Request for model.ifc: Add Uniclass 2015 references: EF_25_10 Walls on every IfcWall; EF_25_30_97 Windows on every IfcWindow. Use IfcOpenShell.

First a look at what the model holds.

```python
import ifcopenshell

model = ifcopenshell.open("model.ifc")
print(model.schema)
print("classifications:", [c.Name for c in model.by_type("IfcClassification")])
for ifc_class in ("IfcDoor", "IfcRoof", "IfcStair", "IfcWall", "IfcWindow"):
    print(ifc_class, len(model.by_type(ifc_class)))
```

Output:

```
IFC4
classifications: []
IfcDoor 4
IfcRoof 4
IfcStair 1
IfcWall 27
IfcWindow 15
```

```python
import ifcopenshell
import ifcopenshell.api.classification

model = ifcopenshell.open("model.ifc")

system = ifcopenshell.api.classification.add_classification(model, classification="Uniclass 2015")

codes = {
    "IfcWall": ("EF_25_10", "Walls"),
    "IfcWindow": ("EF_25_30_97", "Windows"),
}
for ifc_class, (code, name) in codes.items():
    products = model.by_type(ifc_class)
    ifcopenshell.api.classification.add_reference(
        model, products=products, classification=system, identification=code, name=name
    )
    print(code, len(products))

model.write("model-out.ifc")
```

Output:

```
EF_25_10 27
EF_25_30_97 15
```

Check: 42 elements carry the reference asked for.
